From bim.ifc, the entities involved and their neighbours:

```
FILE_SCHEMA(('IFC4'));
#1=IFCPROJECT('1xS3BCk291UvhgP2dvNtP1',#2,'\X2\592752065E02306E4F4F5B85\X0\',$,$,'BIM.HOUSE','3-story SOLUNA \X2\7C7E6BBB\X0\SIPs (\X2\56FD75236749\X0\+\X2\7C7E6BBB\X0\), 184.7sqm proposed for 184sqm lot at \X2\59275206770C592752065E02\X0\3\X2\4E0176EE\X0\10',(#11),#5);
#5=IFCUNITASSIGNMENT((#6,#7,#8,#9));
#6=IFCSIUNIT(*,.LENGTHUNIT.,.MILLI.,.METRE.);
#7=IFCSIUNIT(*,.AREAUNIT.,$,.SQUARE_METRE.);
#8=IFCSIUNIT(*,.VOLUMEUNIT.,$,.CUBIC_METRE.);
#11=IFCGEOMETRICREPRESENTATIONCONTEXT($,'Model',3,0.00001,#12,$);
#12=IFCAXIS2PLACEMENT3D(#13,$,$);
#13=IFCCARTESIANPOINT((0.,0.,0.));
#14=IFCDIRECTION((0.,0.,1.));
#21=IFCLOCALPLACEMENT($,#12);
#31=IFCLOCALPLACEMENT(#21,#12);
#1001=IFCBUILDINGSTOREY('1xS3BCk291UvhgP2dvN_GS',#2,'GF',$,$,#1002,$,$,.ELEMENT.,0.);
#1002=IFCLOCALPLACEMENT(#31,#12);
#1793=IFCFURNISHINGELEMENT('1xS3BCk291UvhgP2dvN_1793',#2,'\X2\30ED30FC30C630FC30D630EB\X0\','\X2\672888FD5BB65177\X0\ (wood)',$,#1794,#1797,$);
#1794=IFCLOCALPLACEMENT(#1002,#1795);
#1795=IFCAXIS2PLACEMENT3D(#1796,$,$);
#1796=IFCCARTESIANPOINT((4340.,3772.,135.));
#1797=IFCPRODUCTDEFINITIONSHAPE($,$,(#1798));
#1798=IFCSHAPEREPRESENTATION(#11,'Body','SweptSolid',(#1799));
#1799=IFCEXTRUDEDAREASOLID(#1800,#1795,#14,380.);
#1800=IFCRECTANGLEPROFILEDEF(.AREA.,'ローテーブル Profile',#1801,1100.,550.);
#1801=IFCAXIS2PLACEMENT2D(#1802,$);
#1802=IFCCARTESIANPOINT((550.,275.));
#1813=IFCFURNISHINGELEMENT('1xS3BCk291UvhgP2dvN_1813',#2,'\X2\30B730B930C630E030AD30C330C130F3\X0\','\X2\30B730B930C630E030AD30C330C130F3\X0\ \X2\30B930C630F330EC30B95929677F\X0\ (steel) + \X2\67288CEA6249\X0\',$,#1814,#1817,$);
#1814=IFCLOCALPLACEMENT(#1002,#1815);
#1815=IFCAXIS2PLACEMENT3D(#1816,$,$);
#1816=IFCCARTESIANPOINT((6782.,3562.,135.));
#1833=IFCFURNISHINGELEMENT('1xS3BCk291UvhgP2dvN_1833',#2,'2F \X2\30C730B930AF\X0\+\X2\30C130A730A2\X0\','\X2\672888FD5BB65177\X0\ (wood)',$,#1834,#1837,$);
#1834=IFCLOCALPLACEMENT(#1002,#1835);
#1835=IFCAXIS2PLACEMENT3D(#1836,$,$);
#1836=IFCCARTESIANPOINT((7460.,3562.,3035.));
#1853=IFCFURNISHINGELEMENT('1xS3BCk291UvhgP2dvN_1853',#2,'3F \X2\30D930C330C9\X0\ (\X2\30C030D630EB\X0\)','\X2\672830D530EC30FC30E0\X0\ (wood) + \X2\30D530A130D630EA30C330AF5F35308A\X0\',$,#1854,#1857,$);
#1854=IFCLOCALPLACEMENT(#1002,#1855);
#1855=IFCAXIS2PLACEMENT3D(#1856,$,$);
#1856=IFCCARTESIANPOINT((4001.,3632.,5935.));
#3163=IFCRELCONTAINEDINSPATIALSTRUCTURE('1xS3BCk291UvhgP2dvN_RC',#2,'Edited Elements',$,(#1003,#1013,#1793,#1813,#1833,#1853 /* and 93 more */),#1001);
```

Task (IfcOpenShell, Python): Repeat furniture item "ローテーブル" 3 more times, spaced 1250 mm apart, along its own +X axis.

```python
import ifcopenshell
import ifcopenshell.api.geometry
import ifcopenshell.api.root
import ifcopenshell.util.element
import ifcopenshell.util.placement
import ifcopenshell.util.unit

model = ifcopenshell.open("bim.ifc")
unit_scale = ifcopenshell.util.unit.calculate_unit_scale(model)


def reuse_history(source, copy):
    """copy_class also copies each property set's owner history, people and application; keep the originals."""
    for rel in copy.IsDefinedBy:
        if rel.is_a("IfcRelDefinesByProperties") and (history := rel.RelatingPropertyDefinition.OwnerHistory):
            rel.RelatingPropertyDefinition.OwnerHistory = source.OwnerHistory
            ifcopenshell.util.element.remove_deep2(model, history)


source = model.by_guid("1xS3BCk291UvhgP2dvN_1793")
base = ifcopenshell.util.placement.get_local_placement(source.ObjectPlacement)
step = base[:3, 0] * 1.25 / unit_scale

for i in range(1, 4):
    copy = ifcopenshell.api.root.copy_class(model, product=source)
    copy.Representation = ifcopenshell.util.element.copy_deep(
        model, source.Representation, exclude=["IfcGeometricRepresentationContext", "IfcRepresentationMap"]
    )
    reuse_history(source, copy)
    matrix = base.copy()
    matrix[:3, 3] += i * step
    print("added at", matrix[:3, 3].round(3) + 0.0)
    ifcopenshell.api.geometry.edit_object_placement(model, product=copy, matrix=matrix, is_si=False)

model.write("bim_v2.ifc")
```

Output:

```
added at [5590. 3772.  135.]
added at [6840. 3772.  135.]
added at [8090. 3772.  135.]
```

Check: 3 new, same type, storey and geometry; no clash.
